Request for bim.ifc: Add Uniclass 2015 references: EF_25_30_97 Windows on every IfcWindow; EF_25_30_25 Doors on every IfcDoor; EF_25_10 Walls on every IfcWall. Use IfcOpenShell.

First a look at what the model holds.

```python
import ifcopenshell

model = ifcopenshell.open("bim.ifc")
print(model.schema)
print("classifications:", [c.Name for c in model.by_type("IfcClassification")])
for ifc_class in ("IfcDoor", "IfcRoof", "IfcStair", "IfcWall", "IfcWindow"):
    print(ifc_class, len(model.by_type(ifc_class)))
```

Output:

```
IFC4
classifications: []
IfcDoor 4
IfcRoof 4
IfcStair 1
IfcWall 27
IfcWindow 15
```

```python
import ifcopenshell
import ifcopenshell.api.classification

model = ifcopenshell.open("bim.ifc")

system = ifcopenshell.api.classification.add_classification(model, classification="Uniclass 2015")

codes = {
    "IfcWindow": ("EF_25_30_97", "Windows"),
    "IfcDoor": ("EF_25_30_25", "Doors"),
    "IfcWall": ("EF_25_10", "Walls"),
}
for ifc_class, (code, name) in codes.items():
    products = model.by_type(ifc_class)
    ifcopenshell.api.classification.add_reference(
        model, products=products, classification=system, identification=code, name=name
    )
    print(code, len(products))

model.write("bim-out.ifc")
```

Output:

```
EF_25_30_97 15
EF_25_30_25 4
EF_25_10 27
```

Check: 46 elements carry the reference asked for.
